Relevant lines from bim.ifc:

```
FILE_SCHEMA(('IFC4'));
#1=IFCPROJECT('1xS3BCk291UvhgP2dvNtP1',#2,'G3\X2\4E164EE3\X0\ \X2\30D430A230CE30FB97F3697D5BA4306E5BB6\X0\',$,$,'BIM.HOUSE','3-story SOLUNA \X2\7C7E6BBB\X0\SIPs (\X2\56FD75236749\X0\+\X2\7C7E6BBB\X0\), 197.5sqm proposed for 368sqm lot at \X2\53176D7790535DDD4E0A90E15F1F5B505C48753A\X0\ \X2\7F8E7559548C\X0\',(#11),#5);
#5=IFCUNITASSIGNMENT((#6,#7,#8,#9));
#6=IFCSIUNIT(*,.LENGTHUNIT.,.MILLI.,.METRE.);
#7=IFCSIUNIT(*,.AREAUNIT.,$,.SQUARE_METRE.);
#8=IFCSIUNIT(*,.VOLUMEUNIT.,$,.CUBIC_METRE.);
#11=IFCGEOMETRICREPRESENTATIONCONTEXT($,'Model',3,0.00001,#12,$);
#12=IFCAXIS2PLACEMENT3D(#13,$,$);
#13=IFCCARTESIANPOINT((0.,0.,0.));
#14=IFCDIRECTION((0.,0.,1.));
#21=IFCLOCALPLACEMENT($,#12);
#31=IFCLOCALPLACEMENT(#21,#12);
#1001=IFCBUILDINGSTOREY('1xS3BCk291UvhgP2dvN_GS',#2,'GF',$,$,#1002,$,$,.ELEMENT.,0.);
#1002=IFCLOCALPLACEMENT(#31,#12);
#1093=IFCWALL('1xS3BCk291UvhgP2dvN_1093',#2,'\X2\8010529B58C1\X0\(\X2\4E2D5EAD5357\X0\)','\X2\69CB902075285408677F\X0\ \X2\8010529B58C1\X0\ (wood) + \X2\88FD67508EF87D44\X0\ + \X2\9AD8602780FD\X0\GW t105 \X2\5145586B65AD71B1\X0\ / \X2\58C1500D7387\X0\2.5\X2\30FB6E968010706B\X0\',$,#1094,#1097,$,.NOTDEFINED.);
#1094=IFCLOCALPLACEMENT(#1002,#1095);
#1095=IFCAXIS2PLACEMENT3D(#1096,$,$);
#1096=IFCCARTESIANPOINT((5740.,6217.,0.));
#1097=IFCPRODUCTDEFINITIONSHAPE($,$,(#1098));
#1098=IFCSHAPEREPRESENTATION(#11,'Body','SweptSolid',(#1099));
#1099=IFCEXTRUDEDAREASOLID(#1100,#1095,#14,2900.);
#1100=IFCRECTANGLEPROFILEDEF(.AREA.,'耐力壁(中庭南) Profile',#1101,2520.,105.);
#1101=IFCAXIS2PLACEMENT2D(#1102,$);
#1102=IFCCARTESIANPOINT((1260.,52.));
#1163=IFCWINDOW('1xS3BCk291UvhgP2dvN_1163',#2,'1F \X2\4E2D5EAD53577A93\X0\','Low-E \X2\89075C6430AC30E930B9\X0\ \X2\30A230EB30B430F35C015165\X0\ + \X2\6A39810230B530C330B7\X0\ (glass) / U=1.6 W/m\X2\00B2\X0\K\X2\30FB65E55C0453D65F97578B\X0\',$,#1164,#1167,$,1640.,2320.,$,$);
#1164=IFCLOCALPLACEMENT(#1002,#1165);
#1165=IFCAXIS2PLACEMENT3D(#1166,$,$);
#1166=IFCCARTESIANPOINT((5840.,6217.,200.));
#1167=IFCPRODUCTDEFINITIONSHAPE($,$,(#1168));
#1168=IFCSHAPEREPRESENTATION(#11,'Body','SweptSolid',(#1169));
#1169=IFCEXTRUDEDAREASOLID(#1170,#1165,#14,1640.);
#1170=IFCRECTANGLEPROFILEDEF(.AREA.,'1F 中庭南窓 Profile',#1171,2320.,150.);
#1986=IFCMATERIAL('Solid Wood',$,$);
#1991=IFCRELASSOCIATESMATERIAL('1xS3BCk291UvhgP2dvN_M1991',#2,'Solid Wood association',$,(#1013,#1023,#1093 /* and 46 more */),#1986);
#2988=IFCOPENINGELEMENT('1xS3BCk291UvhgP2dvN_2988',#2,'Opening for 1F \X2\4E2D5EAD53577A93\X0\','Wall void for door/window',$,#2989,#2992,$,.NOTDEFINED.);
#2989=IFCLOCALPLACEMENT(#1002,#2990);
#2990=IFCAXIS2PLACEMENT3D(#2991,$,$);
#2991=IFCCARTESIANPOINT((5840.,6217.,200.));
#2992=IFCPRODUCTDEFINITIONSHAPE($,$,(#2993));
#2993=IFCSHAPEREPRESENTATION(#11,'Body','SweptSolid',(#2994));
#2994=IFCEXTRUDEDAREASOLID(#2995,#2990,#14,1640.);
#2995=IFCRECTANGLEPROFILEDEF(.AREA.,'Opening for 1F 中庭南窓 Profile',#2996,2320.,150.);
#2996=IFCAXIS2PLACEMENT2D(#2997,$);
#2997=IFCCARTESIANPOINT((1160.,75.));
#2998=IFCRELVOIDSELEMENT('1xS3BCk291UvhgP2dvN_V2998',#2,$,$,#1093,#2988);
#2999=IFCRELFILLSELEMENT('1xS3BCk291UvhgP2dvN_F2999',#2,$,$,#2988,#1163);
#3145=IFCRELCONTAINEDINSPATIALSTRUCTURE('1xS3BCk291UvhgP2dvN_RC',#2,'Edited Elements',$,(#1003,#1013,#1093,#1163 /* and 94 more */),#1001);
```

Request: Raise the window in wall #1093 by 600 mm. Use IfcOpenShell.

```python
import numpy as np
import ifcopenshell
import ifcopenshell.api.geometry
import ifcopenshell.util.placement
import ifcopenshell.util.unit

model = ifcopenshell.open("bim.ifc")
unit_scale = ifcopenshell.util.unit.calculate_unit_scale(model)

window = model.by_id(1163)
opening = window.FillsVoids[0].RelatingOpeningElement
dz = 0.6 / unit_scale

shift = np.array([0.0, 0.0, dz])
# The window is not placed relative to its opening, so move both.
for product in (opening, window):
    matrix = ifcopenshell.util.placement.get_local_placement(product.ObjectPlacement)
    matrix[:3, 3] += shift
    ifcopenshell.api.geometry.edit_object_placement(model, product=product, matrix=matrix, is_si=False)

print(f"moved by {dz * unit_scale:+.3f} m")

model.write("bim_edited.ifc")
```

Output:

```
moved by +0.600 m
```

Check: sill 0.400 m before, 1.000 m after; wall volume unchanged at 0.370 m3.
